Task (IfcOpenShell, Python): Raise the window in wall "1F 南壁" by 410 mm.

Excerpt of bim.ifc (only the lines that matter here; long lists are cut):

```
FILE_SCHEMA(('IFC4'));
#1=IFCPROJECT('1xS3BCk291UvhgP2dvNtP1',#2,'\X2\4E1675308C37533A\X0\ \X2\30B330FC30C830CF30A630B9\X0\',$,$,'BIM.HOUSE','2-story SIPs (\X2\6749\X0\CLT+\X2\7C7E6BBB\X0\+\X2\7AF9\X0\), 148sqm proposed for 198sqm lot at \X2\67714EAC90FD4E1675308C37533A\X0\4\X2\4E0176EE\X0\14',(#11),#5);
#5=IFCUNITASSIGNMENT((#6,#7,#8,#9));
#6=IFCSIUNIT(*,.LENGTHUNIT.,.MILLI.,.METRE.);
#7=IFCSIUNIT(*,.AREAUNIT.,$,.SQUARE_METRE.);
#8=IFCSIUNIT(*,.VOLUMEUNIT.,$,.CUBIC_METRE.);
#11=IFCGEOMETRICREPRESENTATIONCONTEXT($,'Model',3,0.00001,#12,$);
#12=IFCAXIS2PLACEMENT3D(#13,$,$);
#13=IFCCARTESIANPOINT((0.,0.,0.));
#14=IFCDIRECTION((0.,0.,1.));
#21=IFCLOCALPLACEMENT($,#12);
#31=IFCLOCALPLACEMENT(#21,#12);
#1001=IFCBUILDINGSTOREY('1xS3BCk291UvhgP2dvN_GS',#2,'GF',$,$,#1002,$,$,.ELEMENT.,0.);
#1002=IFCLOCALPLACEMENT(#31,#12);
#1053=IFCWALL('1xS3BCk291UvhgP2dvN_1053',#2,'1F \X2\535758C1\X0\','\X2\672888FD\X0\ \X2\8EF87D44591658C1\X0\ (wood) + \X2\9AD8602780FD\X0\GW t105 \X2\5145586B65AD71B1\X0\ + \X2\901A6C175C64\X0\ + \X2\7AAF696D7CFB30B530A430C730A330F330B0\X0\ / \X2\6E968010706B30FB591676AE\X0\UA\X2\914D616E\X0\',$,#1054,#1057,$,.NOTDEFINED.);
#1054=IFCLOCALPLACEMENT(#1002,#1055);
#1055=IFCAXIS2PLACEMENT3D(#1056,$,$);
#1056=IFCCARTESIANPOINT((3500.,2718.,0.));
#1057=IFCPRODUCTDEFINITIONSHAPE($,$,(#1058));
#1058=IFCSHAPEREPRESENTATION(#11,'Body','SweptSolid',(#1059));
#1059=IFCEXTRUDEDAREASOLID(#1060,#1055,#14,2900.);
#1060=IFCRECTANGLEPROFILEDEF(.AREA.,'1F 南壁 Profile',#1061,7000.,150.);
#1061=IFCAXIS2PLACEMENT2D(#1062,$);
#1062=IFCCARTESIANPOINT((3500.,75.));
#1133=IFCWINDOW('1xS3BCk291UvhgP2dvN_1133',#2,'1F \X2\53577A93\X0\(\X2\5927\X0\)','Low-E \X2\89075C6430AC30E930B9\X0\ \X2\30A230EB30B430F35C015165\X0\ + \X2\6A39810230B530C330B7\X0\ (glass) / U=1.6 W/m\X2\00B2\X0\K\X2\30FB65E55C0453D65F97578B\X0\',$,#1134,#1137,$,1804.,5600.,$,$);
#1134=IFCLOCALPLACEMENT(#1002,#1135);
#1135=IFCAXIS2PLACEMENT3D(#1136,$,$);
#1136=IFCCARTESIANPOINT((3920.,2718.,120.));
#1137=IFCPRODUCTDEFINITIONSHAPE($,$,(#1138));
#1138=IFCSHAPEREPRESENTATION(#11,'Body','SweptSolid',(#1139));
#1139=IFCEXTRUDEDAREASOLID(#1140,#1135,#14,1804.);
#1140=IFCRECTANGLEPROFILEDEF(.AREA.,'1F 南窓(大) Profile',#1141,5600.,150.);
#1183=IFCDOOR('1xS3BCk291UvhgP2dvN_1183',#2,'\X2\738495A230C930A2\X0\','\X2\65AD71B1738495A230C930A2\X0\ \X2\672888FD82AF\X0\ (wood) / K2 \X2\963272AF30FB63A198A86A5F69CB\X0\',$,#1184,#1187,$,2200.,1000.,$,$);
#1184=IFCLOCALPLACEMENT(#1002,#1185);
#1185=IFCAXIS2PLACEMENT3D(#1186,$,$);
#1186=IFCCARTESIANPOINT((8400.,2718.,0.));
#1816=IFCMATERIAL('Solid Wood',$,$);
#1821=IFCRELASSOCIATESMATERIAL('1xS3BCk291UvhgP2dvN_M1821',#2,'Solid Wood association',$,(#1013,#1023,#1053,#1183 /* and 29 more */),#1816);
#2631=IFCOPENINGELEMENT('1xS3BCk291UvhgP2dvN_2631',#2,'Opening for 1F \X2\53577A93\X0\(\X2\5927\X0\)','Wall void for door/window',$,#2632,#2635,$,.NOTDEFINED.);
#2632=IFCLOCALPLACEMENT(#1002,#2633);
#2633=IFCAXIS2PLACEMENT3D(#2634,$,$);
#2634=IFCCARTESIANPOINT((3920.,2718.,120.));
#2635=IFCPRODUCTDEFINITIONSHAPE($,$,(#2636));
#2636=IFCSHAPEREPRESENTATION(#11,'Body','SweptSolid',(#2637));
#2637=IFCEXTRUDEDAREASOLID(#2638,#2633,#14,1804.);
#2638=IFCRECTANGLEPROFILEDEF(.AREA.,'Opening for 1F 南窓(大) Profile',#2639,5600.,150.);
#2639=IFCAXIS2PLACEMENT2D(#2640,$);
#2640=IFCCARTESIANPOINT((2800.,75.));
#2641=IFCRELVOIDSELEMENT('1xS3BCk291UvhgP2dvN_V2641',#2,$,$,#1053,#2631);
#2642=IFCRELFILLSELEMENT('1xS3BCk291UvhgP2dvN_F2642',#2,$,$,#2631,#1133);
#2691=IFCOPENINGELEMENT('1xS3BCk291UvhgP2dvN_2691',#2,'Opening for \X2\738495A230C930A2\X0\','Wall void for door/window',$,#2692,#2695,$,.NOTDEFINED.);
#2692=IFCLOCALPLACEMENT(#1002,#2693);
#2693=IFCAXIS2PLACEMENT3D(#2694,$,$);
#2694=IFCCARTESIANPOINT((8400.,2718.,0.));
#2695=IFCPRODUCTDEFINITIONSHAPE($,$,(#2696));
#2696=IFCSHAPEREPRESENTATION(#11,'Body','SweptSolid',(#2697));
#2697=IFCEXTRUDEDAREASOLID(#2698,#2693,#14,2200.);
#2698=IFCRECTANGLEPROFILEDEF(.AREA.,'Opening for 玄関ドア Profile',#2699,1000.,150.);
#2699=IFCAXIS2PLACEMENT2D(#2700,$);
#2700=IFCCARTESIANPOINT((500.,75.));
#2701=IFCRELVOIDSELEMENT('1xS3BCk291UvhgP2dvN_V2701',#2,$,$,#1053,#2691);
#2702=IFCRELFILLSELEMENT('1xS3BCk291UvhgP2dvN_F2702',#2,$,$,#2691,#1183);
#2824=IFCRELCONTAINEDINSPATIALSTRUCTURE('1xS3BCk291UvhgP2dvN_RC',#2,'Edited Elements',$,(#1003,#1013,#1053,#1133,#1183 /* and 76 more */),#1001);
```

```python
import numpy as np
import ifcopenshell
import ifcopenshell.api.geometry
import ifcopenshell.util.placement
import ifcopenshell.util.unit

model = ifcopenshell.open("bim.ifc")
unit_scale = ifcopenshell.util.unit.calculate_unit_scale(model)

window = model.by_guid("1xS3BCk291UvhgP2dvN_1133")
opening = window.FillsVoids[0].RelatingOpeningElement
dz = 410.0

shift = np.array([0.0, 0.0, dz])
# The window is not placed relative to its opening, so move both.
for product in (opening, window):
    matrix = ifcopenshell.util.placement.get_local_placement(product.ObjectPlacement)
    matrix[:3, 3] += shift
    ifcopenshell.api.geometry.edit_object_placement(model, product=product, matrix=matrix, is_si=False)

print(f"moved by {dz * unit_scale:+.3f} m")

model.write("bim_edited.ifc")
```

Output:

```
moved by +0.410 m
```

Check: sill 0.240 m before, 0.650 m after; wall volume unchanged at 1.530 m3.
